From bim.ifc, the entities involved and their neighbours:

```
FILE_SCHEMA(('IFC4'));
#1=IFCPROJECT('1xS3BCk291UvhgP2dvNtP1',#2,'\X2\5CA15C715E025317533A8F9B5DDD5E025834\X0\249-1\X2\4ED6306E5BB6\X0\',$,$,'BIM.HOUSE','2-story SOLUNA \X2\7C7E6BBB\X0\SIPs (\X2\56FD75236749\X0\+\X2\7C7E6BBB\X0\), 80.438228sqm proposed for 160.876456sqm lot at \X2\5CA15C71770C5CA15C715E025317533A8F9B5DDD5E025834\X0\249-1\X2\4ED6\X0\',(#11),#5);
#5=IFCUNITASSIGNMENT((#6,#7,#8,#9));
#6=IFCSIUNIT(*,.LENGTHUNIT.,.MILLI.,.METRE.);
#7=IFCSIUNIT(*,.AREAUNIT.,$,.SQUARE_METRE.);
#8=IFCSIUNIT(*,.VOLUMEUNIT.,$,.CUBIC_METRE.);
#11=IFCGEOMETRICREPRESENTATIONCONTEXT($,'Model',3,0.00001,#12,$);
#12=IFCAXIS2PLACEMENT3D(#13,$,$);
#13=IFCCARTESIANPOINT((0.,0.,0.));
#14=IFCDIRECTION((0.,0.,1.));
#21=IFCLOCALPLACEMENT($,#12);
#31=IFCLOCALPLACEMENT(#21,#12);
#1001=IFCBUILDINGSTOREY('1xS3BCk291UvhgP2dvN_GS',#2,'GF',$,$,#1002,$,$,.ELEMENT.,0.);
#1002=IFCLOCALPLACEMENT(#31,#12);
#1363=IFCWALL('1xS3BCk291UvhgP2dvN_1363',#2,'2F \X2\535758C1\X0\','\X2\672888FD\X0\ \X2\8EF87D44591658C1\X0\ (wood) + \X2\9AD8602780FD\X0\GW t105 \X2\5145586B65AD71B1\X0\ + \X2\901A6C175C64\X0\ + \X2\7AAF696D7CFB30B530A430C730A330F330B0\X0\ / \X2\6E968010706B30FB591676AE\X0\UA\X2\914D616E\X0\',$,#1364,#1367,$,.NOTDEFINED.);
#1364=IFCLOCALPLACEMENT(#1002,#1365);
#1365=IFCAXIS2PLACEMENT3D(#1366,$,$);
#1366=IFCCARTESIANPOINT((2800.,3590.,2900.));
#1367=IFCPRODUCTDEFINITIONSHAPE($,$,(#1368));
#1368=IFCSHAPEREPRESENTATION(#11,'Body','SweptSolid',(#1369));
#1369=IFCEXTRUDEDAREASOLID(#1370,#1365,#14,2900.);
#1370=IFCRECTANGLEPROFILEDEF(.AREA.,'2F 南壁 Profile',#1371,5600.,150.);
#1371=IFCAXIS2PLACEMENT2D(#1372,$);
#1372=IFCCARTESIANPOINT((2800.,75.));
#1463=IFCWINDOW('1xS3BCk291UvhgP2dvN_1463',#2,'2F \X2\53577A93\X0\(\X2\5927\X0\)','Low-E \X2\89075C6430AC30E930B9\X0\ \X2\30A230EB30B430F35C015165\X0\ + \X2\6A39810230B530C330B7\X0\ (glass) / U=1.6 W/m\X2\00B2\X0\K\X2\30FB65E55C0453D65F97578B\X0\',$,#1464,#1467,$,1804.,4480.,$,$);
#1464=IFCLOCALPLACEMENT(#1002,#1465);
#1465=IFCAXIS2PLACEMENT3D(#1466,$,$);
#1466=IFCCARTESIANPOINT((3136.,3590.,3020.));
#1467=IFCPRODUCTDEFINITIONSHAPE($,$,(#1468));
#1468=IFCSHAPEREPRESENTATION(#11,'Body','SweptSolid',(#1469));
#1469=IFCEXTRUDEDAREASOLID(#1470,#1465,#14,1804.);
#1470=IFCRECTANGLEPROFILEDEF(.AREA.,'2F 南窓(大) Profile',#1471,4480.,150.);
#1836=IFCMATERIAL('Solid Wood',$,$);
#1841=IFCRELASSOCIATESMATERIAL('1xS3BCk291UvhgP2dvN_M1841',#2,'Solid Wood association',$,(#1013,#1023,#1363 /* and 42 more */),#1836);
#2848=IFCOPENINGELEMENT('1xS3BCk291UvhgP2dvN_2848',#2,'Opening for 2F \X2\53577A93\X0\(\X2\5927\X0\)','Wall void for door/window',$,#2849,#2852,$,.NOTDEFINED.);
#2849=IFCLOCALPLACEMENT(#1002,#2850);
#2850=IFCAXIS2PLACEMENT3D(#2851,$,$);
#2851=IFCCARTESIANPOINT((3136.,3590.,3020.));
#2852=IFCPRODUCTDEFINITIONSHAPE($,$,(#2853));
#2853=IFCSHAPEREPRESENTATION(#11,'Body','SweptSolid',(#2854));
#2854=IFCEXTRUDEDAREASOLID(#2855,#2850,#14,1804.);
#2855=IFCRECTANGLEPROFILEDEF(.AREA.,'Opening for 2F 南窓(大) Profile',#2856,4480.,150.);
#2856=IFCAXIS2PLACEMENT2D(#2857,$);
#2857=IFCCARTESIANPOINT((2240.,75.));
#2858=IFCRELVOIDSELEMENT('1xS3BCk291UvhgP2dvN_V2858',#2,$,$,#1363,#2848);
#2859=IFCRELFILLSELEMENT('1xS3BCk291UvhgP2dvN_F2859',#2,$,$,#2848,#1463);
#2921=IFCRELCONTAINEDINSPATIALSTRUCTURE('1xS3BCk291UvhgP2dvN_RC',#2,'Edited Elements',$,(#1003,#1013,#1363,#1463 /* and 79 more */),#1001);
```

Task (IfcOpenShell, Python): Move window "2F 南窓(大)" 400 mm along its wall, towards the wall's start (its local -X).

```python
import ifcopenshell
import ifcopenshell.api.geometry
import ifcopenshell.util.placement
import ifcopenshell.util.unit

model = ifcopenshell.open("bim.ifc")
unit_scale = ifcopenshell.util.unit.calculate_unit_scale(model)

window = model.by_guid("1xS3BCk291UvhgP2dvN_1463")
opening = window.FillsVoids[0].RelatingOpeningElement
wall = opening.VoidsElements[0].RelatingBuildingElement

wall_matrix = ifcopenshell.util.placement.get_local_placement(wall.ObjectPlacement)
shift = wall_matrix[:3, 0] * -0.4 / unit_scale
before = ifcopenshell.util.placement.get_local_placement(window.ObjectPlacement)[:3, 3].copy()

# The window is not placed relative to its opening, so move both.
for product in (opening, window):
    matrix = ifcopenshell.util.placement.get_local_placement(product.ObjectPlacement)
    matrix[:3, 3] += shift
    ifcopenshell.api.geometry.edit_object_placement(model, product=product, matrix=matrix, is_si=False)

after = ifcopenshell.util.placement.get_local_placement(window.ObjectPlacement)[:3, 3]
print("window moved by", (after - before).round(3) + 0.0)

model.write("bim_rev.ifc")
```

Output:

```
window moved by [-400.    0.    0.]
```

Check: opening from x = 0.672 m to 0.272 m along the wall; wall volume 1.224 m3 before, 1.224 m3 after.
